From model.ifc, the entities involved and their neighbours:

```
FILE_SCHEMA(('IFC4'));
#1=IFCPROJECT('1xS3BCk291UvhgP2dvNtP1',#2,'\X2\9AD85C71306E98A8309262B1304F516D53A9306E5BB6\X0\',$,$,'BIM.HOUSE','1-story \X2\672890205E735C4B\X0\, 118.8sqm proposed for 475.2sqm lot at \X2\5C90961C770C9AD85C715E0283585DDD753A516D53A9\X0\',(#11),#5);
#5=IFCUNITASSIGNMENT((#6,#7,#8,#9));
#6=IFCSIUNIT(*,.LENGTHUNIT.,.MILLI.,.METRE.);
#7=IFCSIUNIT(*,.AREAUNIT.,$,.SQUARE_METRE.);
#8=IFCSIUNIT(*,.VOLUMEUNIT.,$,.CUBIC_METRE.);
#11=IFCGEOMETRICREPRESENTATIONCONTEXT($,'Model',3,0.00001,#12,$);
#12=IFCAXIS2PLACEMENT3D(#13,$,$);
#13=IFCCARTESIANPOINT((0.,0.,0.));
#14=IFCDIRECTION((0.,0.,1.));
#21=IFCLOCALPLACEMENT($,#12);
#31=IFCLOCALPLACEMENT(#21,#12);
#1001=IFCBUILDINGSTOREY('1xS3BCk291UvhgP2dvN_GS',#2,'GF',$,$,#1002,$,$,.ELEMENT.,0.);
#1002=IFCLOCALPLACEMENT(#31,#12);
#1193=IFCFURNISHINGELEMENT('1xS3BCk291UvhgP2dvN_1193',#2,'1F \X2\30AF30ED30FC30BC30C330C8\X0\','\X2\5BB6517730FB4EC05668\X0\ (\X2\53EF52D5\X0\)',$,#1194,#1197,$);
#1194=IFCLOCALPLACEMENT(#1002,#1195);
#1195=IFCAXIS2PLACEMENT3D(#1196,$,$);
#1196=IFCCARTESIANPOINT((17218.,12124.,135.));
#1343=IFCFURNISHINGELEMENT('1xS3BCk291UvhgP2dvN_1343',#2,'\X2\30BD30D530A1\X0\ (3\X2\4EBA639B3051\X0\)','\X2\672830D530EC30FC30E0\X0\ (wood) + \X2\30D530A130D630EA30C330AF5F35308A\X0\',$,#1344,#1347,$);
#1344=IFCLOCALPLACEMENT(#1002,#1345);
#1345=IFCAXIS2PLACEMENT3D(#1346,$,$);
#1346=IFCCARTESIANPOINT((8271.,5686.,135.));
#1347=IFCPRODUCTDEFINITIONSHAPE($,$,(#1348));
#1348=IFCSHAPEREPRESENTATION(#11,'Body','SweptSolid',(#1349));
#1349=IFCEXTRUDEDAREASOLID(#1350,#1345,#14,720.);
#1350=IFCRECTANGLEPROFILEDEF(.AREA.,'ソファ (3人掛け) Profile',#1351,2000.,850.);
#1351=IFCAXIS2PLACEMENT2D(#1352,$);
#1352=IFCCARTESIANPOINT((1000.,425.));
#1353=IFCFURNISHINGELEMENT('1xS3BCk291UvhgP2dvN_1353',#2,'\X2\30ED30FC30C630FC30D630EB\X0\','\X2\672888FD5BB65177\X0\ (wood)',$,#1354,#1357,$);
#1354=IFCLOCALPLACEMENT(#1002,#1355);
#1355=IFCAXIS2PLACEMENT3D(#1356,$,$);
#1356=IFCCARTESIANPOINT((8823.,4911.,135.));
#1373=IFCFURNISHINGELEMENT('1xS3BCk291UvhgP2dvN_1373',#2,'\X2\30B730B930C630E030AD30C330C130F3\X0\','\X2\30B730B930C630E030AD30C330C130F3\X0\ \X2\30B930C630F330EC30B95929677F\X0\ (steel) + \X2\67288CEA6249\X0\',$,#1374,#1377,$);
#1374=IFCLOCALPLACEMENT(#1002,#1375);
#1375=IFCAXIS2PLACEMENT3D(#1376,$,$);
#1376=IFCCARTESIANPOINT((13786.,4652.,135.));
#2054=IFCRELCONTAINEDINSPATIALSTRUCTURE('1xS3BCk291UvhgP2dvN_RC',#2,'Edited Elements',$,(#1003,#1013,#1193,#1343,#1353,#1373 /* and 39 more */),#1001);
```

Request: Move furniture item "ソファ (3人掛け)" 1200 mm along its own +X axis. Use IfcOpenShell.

```python
import ifcopenshell
import ifcopenshell.api.geometry
import ifcopenshell.util.placement
import ifcopenshell.util.unit

model = ifcopenshell.open("model.ifc")
unit_scale = ifcopenshell.util.unit.calculate_unit_scale(model)

item = model.by_guid("1xS3BCk291UvhgP2dvN_1343")
matrix = ifcopenshell.util.placement.get_local_placement(item.ObjectPlacement)
matrix[:3, 3] += matrix[:3, 0] * 1.2 / unit_scale
ifcopenshell.api.geometry.edit_object_placement(model, product=item, matrix=matrix, is_si=False)

print(ifcopenshell.util.placement.get_local_placement(item.ObjectPlacement).round(3) + 0.0)

model.write("model_updated.ifc")
```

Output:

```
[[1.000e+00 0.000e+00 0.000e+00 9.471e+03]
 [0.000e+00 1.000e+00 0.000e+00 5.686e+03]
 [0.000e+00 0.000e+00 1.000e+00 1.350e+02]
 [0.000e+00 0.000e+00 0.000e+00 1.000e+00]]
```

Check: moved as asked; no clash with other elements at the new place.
